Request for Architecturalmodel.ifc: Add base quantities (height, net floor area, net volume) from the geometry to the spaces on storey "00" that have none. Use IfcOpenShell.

First a look at what the model holds.

```python
import ifcopenshell
import ifcopenshell.util.element
import ifcopenshell.util.unit

model = ifcopenshell.open("Architecturalmodel.ifc")
print(model.schema)
for unit_type in ("LENGTHUNIT", "AREAUNIT", "VOLUMEUNIT"):
    print(unit_type, ifcopenshell.util.unit.calculate_unit_scale(model, unit_type))
storey = next(s for s in model.by_type("IfcBuildingStorey") if s.Name == "00")
spaces = [e for e in ifcopenshell.util.element.get_decomposition(storey) if e.is_a("IfcSpace")]
for e in sorted(spaces, key=lambda e: e.id()):
    print(e.id(), e.is_a(), e.Name, list(ifcopenshell.util.element.get_psets(e, qtos_only=True)), sep=" | ")
```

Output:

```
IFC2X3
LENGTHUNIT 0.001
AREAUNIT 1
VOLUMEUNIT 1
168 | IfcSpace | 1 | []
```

```python
import ifcopenshell
import ifcopenshell.api.pset
import ifcopenshell.geom
import ifcopenshell.util.element
import ifcopenshell.util.shape
import ifcopenshell.util.unit

model = ifcopenshell.open("Architecturalmodel.ifc")
unit_scale = ifcopenshell.util.unit.calculate_unit_scale(model)
area_scale = ifcopenshell.util.unit.calculate_unit_scale(model, "AREAUNIT")
volume_scale = ifcopenshell.util.unit.calculate_unit_scale(model, "VOLUMEUNIT")
settings = ifcopenshell.geom.settings()

storey = next(s for s in model.by_type("IfcBuildingStorey") if s.Name == "00")
spaces = [e for e in ifcopenshell.util.element.get_decomposition(storey) if e.is_a("IfcSpace")]

for e in sorted(spaces, key=lambda e: e.id()):
    if ifcopenshell.util.element.get_psets(e, qtos_only=True, should_inherit=False):
        continue
    # Geometry comes back in metres, in the element's own axes.
    shape = ifcopenshell.geom.create_shape(settings, e)
    values = {
        "Height": ifcopenshell.util.shape.get_z(shape.geometry) / unit_scale,
        "NetFloorArea": ifcopenshell.util.shape.get_footprint_area(shape.geometry) / area_scale,
        "NetVolume": ifcopenshell.util.shape.get_volume(shape.geometry) / volume_scale,
    }
    qto = ifcopenshell.api.pset.add_qto(model, product=e, name="BaseQuantities")
    ifcopenshell.api.pset.edit_qto(model, qto=qto, properties=values)
    print(e.id(), {k: round(v, 3) for k, v in values.items()})

model.write("Architecturalmodel-out.ifc")
```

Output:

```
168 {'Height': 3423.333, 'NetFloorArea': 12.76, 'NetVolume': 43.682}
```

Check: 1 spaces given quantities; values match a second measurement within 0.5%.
